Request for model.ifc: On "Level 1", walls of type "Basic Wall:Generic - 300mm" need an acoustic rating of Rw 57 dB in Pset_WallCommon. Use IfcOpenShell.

First a look at what the model holds.

```python
import ifcopenshell
import ifcopenshell.util.element

model = ifcopenshell.open("model.ifc")
print(model.schema)
storey = next(s for s in model.by_type("IfcBuildingStorey") if s.Name == "Level 1")
walls = [e for e in ifcopenshell.util.element.get_decomposition(storey) if e.is_a("IfcWall")]
seen = {}
for e in walls:
    element_type = ifcopenshell.util.element.get_type(e)
    key = (element_type.Name if element_type != e and element_type else None, ifcopenshell.util.element.get_pset(e, "Pset_WallCommon", "AcousticRating"))
    seen[key] = seen.get(key, 0) + 1
for (name, value), count in sorted(seen.items(), key=str):
    print(count, "x", name, "|", value)
```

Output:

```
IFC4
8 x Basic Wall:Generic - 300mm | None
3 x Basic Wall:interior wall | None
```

```python
import ifcopenshell
import ifcopenshell.api.pset
import ifcopenshell.util.element

model = ifcopenshell.open("model.ifc")

storey = next(s for s in model.by_type("IfcBuildingStorey") if s.Name == "Level 1")
walls = [e for e in ifcopenshell.util.element.get_decomposition(storey) if e.is_a("IfcWall")]

count = 0
for e in walls:
    element_type = ifcopenshell.util.element.get_type(e)
    if element_type in (None, e) or element_type.Name != "Basic Wall:Generic - 300mm":
        continue
    # add_pset returns the element's existing set when there is one.
    pset = ifcopenshell.api.pset.add_pset(model, product=e, name="Pset_WallCommon")
    ifcopenshell.api.pset.edit_pset(model, pset=pset, properties={"AcousticRating": "Rw 57 dB"})
    count += 1

print(count, "walls updated")

model.write("model_updated.ifc")
```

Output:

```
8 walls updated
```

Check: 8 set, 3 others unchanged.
